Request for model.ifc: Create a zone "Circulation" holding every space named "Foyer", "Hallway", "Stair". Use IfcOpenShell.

First a look at what the model holds.

```python
import ifcopenshell

model = ifcopenshell.open("model.ifc")
print(model.schema)
seen = {}
for space in model.by_type("IfcSpace"):
    seen[space.LongName] = seen.get(space.LongName, 0) + 1
for name, count in sorted(seen.items(), key=str):
    print(count, "x", name)
print("zones:", [z.Name for z in model.by_type("IfcZone")][:20])
```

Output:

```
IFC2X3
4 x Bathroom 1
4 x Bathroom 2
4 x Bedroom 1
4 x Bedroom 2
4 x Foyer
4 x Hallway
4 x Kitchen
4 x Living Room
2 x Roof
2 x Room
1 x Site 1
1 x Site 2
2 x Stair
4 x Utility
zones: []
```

```python
import ifcopenshell
import ifcopenshell.api.group
import ifcopenshell.api.root

model = ifcopenshell.open("model.ifc")

names = {"Foyer", "Hallway", "Stair"}
spaces = [s for s in model.by_type("IfcSpace") if s.LongName in names]

zone = ifcopenshell.api.root.create_entity(model, ifc_class="IfcZone", name="Circulation")
ifcopenshell.api.group.assign_group(model, products=spaces, group=zone)
print(len(spaces), "spaces in", zone.Name)

model.write("model_v2.ifc")
```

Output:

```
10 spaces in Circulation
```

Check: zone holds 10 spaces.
